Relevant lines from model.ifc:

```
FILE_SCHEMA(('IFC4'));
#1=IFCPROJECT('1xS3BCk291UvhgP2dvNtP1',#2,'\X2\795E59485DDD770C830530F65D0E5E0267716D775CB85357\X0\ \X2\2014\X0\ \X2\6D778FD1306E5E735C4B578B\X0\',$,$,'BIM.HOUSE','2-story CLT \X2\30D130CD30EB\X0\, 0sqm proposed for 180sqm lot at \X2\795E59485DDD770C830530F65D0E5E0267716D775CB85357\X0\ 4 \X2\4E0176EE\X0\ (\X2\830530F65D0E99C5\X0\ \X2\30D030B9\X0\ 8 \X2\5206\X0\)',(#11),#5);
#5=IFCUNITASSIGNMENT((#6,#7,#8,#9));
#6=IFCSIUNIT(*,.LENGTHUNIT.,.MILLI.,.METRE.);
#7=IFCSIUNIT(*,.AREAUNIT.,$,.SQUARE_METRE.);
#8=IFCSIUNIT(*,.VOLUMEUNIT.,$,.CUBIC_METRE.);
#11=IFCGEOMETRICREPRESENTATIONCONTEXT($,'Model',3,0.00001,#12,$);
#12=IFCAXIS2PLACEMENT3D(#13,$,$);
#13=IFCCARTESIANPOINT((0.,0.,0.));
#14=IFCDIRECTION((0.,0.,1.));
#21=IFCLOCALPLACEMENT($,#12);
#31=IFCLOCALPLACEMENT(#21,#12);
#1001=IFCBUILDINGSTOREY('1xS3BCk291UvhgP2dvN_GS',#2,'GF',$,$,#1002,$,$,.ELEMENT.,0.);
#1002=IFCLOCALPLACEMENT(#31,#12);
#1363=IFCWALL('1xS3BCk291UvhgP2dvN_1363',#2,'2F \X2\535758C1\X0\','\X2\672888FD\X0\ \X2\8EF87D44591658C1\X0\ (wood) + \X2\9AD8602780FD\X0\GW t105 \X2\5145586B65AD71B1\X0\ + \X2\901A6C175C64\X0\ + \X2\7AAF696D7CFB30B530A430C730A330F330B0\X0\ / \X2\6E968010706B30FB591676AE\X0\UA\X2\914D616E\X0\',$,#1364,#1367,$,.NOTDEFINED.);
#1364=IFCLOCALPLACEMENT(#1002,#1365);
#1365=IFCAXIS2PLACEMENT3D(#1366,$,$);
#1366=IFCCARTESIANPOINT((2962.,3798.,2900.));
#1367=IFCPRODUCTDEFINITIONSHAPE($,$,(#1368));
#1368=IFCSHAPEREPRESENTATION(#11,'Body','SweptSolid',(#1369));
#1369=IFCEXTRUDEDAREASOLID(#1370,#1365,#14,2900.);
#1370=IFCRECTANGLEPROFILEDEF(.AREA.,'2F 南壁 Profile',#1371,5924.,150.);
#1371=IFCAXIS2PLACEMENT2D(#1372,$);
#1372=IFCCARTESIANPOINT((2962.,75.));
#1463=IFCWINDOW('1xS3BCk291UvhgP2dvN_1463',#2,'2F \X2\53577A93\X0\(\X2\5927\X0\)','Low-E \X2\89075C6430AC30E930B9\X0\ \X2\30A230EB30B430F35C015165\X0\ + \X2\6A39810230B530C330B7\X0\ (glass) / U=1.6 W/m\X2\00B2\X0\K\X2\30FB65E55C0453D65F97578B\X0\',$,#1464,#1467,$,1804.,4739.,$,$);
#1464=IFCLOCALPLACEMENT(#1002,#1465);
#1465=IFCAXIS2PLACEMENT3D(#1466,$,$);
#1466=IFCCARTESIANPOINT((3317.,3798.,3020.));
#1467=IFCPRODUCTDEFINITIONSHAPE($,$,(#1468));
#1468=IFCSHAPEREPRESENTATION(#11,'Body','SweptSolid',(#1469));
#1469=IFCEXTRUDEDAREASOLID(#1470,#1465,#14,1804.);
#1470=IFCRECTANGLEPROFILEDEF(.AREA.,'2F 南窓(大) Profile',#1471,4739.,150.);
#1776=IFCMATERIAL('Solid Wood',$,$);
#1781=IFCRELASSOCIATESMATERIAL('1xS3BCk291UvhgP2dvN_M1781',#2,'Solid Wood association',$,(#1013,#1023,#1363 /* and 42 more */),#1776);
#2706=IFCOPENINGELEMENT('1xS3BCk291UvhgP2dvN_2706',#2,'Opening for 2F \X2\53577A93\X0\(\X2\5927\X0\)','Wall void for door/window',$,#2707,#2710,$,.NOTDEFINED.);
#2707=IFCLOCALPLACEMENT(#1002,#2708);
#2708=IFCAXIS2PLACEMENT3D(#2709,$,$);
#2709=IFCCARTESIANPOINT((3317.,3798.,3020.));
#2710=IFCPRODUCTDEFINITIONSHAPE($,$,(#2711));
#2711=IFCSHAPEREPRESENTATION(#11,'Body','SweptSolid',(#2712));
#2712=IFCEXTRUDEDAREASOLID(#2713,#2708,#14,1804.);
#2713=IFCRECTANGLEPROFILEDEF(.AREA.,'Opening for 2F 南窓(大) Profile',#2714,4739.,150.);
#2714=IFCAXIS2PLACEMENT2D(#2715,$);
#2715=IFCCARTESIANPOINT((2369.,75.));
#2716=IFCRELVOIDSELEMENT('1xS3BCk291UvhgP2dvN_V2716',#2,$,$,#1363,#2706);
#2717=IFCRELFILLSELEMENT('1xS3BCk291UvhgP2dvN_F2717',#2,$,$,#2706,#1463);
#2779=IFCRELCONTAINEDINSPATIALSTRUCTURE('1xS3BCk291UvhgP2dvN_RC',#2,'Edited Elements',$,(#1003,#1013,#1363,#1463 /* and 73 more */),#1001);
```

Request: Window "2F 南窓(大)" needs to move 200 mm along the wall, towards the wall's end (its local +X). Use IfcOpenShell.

```python
import ifcopenshell
import ifcopenshell.api.geometry
import ifcopenshell.util.placement
import ifcopenshell.util.unit

model = ifcopenshell.open("model.ifc")
unit_scale = ifcopenshell.util.unit.calculate_unit_scale(model)

window = model.by_guid("1xS3BCk291UvhgP2dvN_1463")
opening = window.FillsVoids[0].RelatingOpeningElement
wall = opening.VoidsElements[0].RelatingBuildingElement

wall_matrix = ifcopenshell.util.placement.get_local_placement(wall.ObjectPlacement)
shift = wall_matrix[:3, 0] * 0.2 / unit_scale
before = ifcopenshell.util.placement.get_local_placement(window.ObjectPlacement)[:3, 3].copy()

# The window is not placed relative to its opening, so move both.
for product in (opening, window):
    matrix = ifcopenshell.util.placement.get_local_placement(product.ObjectPlacement)
    matrix[:3, 3] += shift
    ifcopenshell.api.geometry.edit_object_placement(model, product=product, matrix=matrix, is_si=False)

after = ifcopenshell.util.placement.get_local_placement(window.ObjectPlacement)[:3, 3]
print("window moved by", (after - before).round(3) + 0.0)

model.write("model_rev.ifc")
```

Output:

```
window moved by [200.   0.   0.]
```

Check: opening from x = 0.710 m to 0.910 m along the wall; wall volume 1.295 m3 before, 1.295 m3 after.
